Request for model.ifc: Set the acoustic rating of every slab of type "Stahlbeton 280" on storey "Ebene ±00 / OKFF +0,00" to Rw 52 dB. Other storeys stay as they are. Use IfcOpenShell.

First a look at what the model holds.

```python
import ifcopenshell
import ifcopenshell.util.element

model = ifcopenshell.open("model.ifc")
print(model.schema)
storey = next(s for s in model.by_type("IfcBuildingStorey") if s.Name == "Ebene ±00 / OKFF +0,00")
slabs = [e for e in ifcopenshell.util.element.get_decomposition(storey) if e.is_a("IfcSlab")]
seen = {}
for e in slabs:
    element_type = ifcopenshell.util.element.get_type(e)
    key = (element_type.Name if element_type != e and element_type else None, ifcopenshell.util.element.get_pset(e, "Pset_SlabCommon", "AcousticRating"))
    seen[key] = seen.get(key, 0) + 1
for (name, value), count in sorted(seen.items(), key=str):
    print(count, "x", name, "|", value)
```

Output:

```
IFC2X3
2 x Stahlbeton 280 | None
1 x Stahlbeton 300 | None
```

```python
import ifcopenshell
import ifcopenshell.api.pset
import ifcopenshell.util.element

model = ifcopenshell.open("model.ifc")

storey = next(s for s in model.by_type("IfcBuildingStorey") if s.Name == "Ebene ±00 / OKFF +0,00")
slabs = [e for e in ifcopenshell.util.element.get_decomposition(storey) if e.is_a("IfcSlab")]

count = 0
for e in slabs:
    element_type = ifcopenshell.util.element.get_type(e)
    if element_type in (None, e) or element_type.Name != "Stahlbeton 280":
        continue
    # add_pset returns the element's existing set when there is one.
    pset = ifcopenshell.api.pset.add_pset(model, product=e, name="Pset_SlabCommon")
    ifcopenshell.api.pset.edit_pset(model, pset=pset, properties={"AcousticRating": "Rw 52 dB"})
    count += 1

print(count, "slabs updated")

model.write("model-out.ifc")
```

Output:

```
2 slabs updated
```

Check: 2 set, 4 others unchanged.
